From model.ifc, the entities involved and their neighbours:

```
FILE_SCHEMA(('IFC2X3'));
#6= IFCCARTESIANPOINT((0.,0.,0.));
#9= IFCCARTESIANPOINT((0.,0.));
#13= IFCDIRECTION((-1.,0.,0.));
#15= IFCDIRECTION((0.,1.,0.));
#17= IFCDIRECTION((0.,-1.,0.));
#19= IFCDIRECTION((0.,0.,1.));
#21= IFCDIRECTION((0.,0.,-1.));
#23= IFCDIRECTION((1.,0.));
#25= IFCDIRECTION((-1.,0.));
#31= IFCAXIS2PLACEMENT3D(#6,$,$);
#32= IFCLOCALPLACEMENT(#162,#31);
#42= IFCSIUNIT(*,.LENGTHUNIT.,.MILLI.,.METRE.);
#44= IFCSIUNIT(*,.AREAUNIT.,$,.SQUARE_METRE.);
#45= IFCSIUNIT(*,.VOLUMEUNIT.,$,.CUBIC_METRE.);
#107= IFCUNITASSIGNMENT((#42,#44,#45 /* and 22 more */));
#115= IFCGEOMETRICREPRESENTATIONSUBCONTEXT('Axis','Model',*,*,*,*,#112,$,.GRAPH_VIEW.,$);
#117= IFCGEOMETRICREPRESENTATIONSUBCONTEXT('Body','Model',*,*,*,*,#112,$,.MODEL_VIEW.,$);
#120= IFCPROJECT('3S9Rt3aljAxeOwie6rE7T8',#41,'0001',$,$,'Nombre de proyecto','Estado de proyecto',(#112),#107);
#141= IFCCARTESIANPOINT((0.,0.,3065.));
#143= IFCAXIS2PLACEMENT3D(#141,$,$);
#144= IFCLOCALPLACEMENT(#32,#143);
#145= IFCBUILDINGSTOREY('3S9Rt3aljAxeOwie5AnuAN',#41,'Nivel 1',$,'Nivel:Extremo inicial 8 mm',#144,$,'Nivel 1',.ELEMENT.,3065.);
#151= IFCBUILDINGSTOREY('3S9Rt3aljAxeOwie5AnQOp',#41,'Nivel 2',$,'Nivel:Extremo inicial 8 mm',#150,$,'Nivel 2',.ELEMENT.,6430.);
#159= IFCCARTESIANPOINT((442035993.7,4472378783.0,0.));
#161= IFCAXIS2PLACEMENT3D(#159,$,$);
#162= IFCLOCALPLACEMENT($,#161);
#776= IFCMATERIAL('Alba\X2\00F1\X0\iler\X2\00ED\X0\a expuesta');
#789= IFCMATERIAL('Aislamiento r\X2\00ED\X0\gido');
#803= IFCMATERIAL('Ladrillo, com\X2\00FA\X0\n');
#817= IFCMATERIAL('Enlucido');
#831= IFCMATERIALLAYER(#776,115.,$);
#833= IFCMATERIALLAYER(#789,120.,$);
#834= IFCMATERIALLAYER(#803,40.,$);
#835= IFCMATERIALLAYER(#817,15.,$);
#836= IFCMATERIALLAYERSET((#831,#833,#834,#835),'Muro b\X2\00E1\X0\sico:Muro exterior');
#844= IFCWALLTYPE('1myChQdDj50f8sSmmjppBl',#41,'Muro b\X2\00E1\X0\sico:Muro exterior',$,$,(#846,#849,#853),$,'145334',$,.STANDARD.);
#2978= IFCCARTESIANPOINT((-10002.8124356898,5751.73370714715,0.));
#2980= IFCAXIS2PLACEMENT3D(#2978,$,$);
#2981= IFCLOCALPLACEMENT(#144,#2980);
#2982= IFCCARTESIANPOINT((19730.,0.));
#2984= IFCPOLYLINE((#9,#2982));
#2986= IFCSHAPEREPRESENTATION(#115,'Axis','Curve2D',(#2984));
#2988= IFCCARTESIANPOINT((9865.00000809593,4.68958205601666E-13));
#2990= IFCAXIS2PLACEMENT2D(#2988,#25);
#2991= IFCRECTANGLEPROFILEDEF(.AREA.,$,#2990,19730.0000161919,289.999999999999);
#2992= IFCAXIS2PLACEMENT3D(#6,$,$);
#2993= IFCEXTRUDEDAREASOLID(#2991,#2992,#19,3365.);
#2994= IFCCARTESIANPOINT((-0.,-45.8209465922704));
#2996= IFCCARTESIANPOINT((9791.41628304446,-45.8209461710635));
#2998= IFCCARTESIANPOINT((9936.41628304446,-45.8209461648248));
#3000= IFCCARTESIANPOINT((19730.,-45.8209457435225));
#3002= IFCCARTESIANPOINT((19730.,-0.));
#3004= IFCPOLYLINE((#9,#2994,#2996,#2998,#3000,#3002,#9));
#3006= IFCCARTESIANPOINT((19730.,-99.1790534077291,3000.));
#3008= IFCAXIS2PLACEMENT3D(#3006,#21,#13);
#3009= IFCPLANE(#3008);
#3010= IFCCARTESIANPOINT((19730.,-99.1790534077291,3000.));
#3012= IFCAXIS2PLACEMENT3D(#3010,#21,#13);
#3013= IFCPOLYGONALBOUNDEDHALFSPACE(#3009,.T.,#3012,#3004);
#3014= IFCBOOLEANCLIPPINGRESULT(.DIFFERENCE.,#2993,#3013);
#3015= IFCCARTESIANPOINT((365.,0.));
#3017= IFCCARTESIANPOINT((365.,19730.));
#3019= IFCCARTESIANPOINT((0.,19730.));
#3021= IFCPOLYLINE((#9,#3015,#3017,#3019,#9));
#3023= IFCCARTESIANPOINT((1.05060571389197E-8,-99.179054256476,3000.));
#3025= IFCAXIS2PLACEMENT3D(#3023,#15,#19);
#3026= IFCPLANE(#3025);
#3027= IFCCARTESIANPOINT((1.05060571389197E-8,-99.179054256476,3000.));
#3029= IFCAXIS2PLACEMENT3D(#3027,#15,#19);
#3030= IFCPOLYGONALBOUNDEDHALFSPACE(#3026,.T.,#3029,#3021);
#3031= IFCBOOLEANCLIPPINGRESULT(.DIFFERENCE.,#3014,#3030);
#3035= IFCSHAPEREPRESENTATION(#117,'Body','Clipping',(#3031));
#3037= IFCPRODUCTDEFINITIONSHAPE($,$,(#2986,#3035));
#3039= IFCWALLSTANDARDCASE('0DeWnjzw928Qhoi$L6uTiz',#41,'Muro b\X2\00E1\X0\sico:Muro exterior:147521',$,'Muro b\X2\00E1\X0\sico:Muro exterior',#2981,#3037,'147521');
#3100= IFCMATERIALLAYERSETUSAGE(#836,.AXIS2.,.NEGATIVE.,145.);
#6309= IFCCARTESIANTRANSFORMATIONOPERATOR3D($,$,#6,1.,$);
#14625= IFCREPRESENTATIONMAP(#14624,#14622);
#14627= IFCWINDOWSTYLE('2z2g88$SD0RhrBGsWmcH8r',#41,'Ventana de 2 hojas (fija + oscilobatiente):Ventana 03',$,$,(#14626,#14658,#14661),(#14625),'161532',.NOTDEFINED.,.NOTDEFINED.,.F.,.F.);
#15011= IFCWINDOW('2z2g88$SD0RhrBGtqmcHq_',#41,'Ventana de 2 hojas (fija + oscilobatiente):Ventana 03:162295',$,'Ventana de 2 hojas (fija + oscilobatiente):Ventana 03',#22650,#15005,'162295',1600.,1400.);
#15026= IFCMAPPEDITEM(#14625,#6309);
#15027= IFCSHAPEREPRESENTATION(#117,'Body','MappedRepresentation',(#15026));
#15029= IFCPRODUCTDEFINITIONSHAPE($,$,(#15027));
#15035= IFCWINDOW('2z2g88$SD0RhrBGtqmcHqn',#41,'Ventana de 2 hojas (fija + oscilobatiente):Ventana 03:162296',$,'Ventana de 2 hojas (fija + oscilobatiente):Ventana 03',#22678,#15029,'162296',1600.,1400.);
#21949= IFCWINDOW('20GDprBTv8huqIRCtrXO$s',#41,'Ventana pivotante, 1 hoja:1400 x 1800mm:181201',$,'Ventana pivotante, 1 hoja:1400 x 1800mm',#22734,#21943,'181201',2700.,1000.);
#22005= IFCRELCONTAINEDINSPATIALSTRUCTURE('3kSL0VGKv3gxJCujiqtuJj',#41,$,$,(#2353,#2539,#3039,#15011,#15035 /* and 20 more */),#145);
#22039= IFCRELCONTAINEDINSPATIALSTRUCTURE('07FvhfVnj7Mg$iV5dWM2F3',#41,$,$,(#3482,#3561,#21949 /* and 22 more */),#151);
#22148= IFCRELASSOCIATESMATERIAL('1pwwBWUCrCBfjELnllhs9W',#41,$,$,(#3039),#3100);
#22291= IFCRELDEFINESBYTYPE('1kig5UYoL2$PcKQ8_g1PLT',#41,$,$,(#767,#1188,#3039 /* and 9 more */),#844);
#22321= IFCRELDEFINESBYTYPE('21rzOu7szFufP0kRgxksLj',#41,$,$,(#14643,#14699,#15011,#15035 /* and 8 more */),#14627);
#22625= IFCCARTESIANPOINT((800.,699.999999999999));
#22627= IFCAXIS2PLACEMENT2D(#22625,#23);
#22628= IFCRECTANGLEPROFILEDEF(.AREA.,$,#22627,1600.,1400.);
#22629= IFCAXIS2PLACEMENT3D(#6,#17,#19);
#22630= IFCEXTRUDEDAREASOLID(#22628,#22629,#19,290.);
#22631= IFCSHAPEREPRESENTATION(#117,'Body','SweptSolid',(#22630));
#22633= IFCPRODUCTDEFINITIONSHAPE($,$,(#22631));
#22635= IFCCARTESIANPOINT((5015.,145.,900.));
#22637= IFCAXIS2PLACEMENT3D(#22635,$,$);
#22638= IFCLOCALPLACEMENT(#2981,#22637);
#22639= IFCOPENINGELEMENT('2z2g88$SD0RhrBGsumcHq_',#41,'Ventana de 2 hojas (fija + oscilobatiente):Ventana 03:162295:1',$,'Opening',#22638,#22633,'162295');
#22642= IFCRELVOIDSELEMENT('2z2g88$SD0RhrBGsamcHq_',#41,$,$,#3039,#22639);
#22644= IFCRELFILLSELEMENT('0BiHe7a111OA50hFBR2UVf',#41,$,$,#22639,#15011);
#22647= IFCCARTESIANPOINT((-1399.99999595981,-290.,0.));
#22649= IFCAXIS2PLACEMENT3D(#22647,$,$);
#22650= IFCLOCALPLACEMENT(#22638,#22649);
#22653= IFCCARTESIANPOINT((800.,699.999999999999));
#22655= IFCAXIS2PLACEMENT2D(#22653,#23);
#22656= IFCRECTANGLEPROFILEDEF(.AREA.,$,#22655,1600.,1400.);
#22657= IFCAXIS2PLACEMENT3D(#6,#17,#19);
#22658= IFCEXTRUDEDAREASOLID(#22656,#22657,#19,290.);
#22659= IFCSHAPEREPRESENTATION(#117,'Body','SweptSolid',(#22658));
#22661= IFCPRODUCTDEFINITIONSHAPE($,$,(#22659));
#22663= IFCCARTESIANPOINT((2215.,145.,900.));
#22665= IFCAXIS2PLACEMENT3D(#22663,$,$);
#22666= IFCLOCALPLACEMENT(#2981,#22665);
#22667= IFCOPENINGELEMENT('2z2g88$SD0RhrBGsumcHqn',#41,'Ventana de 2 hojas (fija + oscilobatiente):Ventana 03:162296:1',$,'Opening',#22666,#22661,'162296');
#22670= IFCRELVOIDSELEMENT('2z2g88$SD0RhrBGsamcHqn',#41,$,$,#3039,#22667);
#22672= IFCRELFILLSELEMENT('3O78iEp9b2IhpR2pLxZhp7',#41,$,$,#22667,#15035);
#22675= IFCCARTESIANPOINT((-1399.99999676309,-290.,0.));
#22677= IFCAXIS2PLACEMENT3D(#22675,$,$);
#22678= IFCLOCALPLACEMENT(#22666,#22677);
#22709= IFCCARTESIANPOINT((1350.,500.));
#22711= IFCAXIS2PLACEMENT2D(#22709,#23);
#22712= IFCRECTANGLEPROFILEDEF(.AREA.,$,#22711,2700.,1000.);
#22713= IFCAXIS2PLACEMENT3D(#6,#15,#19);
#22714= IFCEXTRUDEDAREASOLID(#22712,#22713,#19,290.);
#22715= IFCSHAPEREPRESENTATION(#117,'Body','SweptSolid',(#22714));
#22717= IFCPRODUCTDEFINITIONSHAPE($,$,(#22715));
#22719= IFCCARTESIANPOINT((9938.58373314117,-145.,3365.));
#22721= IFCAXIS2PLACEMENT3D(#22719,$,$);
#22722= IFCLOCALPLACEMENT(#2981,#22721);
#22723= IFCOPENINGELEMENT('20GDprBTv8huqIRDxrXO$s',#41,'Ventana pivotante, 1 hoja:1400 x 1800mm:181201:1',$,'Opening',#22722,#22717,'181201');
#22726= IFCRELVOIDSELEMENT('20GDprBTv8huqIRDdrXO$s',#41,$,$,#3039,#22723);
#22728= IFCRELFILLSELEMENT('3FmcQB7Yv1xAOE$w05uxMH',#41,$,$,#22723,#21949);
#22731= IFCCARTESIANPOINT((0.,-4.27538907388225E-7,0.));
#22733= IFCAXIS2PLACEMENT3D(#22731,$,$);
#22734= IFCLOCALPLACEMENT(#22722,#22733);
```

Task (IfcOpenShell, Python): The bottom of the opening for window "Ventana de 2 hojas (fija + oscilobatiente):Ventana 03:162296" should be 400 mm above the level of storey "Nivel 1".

```python
import numpy as np
import ifcopenshell
import ifcopenshell.api.geometry
import ifcopenshell.geom
import ifcopenshell.util.element
import ifcopenshell.util.placement
import ifcopenshell.util.shape
import ifcopenshell.util.unit

model = ifcopenshell.open("model.ifc")
unit_scale = ifcopenshell.util.unit.calculate_unit_scale(model)

window = model.by_guid("2z2g88$SD0RhrBGtqmcHqn")
opening = window.FillsVoids[0].RelatingOpeningElement
storey = ifcopenshell.util.element.get_container(window, ifc_class="IfcBuildingStorey")
level = ifcopenshell.util.placement.get_local_placement(storey.ObjectPlacement)[2, 3]

# The opening's origin need not be at the sill, so measure its lowest point.
shape = ifcopenshell.geom.create_shape(ifcopenshell.geom.settings(), opening)
bottom = ifcopenshell.util.shape.get_shape_bottom_elevation(shape, shape.geometry) / unit_scale
dz = level + 400.0 - bottom

shift = np.array([0.0, 0.0, dz])
# The window is placed relative to its opening, so it follows when the opening moves.
matrix = ifcopenshell.util.placement.get_local_placement(opening.ObjectPlacement)
matrix[:3, 3] += shift
ifcopenshell.api.geometry.edit_object_placement(
    model, product=opening, matrix=matrix, is_si=False, should_transform_children=True
)

print(f"moved by {dz * unit_scale:+.3f} m")

model.write("model_edited.ifc")
```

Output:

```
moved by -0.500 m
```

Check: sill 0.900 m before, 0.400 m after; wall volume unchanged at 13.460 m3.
